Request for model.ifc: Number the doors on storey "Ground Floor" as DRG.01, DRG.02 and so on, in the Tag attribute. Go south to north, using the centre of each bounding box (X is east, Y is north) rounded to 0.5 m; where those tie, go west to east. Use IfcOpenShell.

First a look at what the model holds.

```python
import ifcopenshell
import ifcopenshell.util.element
import ifcopenshell.util.placement

model = ifcopenshell.open("model.ifc")
print(model.schema)
storey = next(s for s in model.by_type("IfcBuildingStorey") if s.Name == "Ground Floor")
doors = [e for e in ifcopenshell.util.element.get_decomposition(storey) if e.is_a("IfcDoor")]
for e in sorted(doors, key=lambda e: e.id()):
    origin = ifcopenshell.util.placement.get_local_placement(e.ObjectPlacement)[:3, 3]
    print(e.id(), e.Tag, e.Name, origin.round(2) + 0.0, sep=" | ")
```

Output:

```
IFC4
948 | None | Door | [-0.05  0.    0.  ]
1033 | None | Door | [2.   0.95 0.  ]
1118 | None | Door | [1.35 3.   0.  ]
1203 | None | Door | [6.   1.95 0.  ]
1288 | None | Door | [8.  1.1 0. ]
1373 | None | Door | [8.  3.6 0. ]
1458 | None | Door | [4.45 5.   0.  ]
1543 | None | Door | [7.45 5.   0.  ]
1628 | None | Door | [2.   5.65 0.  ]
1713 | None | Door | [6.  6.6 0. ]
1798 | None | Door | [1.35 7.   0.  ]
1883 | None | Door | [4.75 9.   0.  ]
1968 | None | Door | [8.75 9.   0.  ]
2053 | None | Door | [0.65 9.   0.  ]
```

```python
import ifcopenshell
import ifcopenshell.geom
import ifcopenshell.util.element
import ifcopenshell.util.shape

model = ifcopenshell.open("model.ifc")
settings = ifcopenshell.geom.settings()
settings.set("use-world-coords", True)


def centre(element):
    shape = ifcopenshell.geom.create_shape(settings, element)
    return ifcopenshell.util.shape.get_bbox_centroid(shape.geometry)


storey = next(s for s in model.by_type("IfcBuildingStorey") if s.Name == "Ground Floor")
doors = [e for e in ifcopenshell.util.element.get_decomposition(storey) if e.is_a("IfcDoor")]

# Insertion points can sit at a corner or the storey origin, so sort by the geometry (in metres).
centres = {e: centre(e) for e in doors}
doors.sort(key=lambda e: (round(centres[e][1] / 0.5), centres[e][0]))

for i, e in enumerate(doors, start=1):
    number = f"DRG.{i:02d}"
    e.Tag = number
    print(e.id(), number)

model.write("model_edited.ifc")
```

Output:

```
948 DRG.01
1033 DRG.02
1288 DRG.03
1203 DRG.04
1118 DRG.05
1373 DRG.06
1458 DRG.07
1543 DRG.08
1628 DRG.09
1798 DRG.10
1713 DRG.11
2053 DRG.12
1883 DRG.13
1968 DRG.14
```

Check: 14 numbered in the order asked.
